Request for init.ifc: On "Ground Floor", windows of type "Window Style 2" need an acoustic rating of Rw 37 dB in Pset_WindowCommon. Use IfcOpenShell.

First a look at what the model holds.

```python
import ifcopenshell
import ifcopenshell.util.element

model = ifcopenshell.open("init.ifc")
print(model.schema)
storey = next(s for s in model.by_type("IfcBuildingStorey") if s.Name == "Ground Floor")
windows = [e for e in ifcopenshell.util.element.get_decomposition(storey) if e.is_a("IfcWindow")]
seen = {}
for e in windows:
    element_type = ifcopenshell.util.element.get_type(e)
    key = (element_type.Name if element_type != e and element_type else None, ifcopenshell.util.element.get_pset(e, "Pset_WindowCommon", "AcousticRating"))
    seen[key] = seen.get(key, 0) + 1
for (name, value), count in sorted(seen.items(), key=str):
    print(count, "x", name, "|", value)
```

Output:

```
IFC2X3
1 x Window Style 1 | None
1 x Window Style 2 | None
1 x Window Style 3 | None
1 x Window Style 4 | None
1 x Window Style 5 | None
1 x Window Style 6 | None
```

```python
import ifcopenshell
import ifcopenshell.api.pset
import ifcopenshell.util.element

model = ifcopenshell.open("init.ifc")

storey = next(s for s in model.by_type("IfcBuildingStorey") if s.Name == "Ground Floor")
windows = [e for e in ifcopenshell.util.element.get_decomposition(storey) if e.is_a("IfcWindow")]

count = 0
for e in windows:
    element_type = ifcopenshell.util.element.get_type(e)
    if element_type in (None, e) or element_type.Name != "Window Style 2":
        continue
    # add_pset returns the element's existing set when there is one.
    pset = ifcopenshell.api.pset.add_pset(model, product=e, name="Pset_WindowCommon")
    ifcopenshell.api.pset.edit_pset(model, pset=pset, properties={"AcousticRating": "Rw 37 dB"})
    count += 1

print(count, "windows updated")

model.write("init_updated.ifc")
```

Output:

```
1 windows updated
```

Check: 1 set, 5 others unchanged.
